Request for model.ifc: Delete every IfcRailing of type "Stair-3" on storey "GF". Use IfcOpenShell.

First a look at what the model holds.

```python
import ifcopenshell
import ifcopenshell.util.element

model = ifcopenshell.open("model.ifc")
print(model.schema)
storey = next(s for s in model.by_type("IfcBuildingStorey") if s.Name == "GF")
railings = [e for e in ifcopenshell.util.element.get_decomposition(storey) if e.is_a("IfcRailing")]
seen = {}
for e in railings:
    element_type = ifcopenshell.util.element.get_type(e)
    name = element_type.Name if element_type not in (None, e) else None
    seen[name] = seen.get(name, 0) + 1
for name, count in sorted(seen.items(), key=str):
    print(count, "x", name)
```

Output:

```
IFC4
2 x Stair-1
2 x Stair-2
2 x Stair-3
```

```python
import ifcopenshell
import ifcopenshell.api.root
import ifcopenshell.util.element

model = ifcopenshell.open("model.ifc")

storey = next(s for s in model.by_type("IfcBuildingStorey") if s.Name == "GF")
railings = [e for e in ifcopenshell.util.element.get_decomposition(storey) if e.is_a("IfcRailing")]
targets = [e for e in railings if (t := ifcopenshell.util.element.get_type(e)) not in (None, e) and t.Name == "Stair-3"]

for e in targets:
    ifcopenshell.api.root.remove_product(model, product=e)
print(len(targets), "removed")

model.write("model-out.ifc")
```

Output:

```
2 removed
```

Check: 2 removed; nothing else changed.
